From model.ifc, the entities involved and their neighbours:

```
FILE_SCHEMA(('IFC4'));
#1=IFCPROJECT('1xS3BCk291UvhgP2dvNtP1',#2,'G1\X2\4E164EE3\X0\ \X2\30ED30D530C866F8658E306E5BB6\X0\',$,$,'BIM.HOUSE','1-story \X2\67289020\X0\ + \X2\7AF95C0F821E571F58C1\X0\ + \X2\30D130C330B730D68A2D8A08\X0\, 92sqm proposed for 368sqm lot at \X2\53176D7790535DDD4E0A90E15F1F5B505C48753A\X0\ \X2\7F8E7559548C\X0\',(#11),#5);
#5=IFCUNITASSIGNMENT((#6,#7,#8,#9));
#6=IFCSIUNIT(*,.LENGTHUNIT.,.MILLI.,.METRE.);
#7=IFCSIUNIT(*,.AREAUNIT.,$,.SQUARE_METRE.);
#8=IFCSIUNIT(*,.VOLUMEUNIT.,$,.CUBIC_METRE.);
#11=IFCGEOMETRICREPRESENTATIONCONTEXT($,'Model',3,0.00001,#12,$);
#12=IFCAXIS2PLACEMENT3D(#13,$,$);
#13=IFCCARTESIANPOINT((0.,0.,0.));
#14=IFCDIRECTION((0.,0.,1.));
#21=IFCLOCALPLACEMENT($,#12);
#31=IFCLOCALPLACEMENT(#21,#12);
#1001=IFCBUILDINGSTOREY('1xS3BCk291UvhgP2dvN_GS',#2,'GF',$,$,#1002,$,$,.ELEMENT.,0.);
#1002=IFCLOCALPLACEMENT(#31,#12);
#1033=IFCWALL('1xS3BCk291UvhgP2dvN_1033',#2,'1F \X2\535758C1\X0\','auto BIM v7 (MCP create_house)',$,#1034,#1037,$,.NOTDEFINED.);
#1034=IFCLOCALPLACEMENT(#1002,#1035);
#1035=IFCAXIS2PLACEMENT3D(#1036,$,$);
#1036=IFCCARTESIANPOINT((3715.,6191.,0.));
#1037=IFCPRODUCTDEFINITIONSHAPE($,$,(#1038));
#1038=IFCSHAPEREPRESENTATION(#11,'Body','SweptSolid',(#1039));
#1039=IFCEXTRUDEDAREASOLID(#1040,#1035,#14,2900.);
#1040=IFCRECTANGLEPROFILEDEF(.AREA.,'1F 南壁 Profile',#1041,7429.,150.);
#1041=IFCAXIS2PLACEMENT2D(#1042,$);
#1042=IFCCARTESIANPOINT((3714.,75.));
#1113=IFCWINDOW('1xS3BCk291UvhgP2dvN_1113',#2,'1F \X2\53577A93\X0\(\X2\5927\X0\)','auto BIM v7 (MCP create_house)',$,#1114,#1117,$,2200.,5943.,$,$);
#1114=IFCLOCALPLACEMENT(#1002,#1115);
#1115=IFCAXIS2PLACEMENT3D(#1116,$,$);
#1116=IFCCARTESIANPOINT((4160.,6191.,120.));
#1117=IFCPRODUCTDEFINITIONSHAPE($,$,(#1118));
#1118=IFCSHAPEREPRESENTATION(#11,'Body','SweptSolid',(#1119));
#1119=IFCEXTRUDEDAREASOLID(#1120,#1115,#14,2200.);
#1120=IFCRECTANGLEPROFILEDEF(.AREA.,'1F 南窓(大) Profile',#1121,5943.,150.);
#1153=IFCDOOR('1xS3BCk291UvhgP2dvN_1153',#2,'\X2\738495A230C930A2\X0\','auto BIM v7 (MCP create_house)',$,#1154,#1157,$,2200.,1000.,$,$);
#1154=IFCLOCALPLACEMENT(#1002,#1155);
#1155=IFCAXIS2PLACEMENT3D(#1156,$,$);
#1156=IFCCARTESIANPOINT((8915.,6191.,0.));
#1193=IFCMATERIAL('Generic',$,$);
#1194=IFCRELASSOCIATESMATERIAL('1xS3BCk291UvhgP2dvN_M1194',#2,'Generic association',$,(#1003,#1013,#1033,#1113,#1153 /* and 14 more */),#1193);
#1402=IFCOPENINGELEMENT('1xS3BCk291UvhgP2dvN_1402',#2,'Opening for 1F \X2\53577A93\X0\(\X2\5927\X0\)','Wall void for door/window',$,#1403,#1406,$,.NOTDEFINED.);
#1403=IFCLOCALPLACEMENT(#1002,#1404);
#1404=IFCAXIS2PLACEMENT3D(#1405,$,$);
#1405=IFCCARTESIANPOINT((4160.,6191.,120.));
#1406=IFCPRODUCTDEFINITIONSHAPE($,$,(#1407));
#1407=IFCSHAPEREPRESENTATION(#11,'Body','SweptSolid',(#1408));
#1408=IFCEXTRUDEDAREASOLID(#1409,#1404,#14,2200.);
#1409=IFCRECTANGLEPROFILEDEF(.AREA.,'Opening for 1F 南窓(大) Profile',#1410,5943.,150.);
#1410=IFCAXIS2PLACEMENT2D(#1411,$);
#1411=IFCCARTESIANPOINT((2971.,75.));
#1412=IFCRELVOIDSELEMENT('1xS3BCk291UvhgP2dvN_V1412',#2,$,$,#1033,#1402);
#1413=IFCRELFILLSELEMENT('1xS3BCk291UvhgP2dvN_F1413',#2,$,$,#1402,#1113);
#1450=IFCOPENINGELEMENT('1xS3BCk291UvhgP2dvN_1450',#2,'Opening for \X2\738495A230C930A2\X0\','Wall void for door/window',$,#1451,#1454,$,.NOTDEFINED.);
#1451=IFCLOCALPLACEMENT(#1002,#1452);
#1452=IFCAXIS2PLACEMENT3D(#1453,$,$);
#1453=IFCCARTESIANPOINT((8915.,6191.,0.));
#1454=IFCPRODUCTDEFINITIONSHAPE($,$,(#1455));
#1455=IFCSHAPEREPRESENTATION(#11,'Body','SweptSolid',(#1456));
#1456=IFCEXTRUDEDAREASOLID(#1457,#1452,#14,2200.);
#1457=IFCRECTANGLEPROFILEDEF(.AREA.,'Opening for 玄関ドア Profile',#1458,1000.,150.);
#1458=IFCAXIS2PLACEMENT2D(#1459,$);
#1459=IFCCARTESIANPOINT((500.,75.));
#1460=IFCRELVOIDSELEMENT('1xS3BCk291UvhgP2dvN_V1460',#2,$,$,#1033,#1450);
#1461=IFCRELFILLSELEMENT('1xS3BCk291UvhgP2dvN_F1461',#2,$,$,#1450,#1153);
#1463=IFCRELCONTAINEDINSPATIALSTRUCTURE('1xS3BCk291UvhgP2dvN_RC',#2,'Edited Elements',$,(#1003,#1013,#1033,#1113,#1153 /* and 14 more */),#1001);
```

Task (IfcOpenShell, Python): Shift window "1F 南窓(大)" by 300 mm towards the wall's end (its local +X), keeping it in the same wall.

```python
import ifcopenshell
import ifcopenshell.api.geometry
import ifcopenshell.util.placement

model = ifcopenshell.open("model.ifc")

window = model.by_guid("1xS3BCk291UvhgP2dvN_1113")
opening = window.FillsVoids[0].RelatingOpeningElement
wall = opening.VoidsElements[0].RelatingBuildingElement

wall_matrix = ifcopenshell.util.placement.get_local_placement(wall.ObjectPlacement)
shift = wall_matrix[:3, 0] * 300.0
before = ifcopenshell.util.placement.get_local_placement(window.ObjectPlacement)[:3, 3].copy()

# The window is not placed relative to its opening, so move both.
for product in (opening, window):
    matrix = ifcopenshell.util.placement.get_local_placement(product.ObjectPlacement)
    matrix[:3, 3] += shift
    ifcopenshell.api.geometry.edit_object_placement(model, product=product, matrix=matrix, is_si=False)

after = ifcopenshell.util.placement.get_local_placement(window.ObjectPlacement)[:3, 3]
print("window moved by", (after - before).round(3) + 0.0)

model.write("model_v2.ifc")
```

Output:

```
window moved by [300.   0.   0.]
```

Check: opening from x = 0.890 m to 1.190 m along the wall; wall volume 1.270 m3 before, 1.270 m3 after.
